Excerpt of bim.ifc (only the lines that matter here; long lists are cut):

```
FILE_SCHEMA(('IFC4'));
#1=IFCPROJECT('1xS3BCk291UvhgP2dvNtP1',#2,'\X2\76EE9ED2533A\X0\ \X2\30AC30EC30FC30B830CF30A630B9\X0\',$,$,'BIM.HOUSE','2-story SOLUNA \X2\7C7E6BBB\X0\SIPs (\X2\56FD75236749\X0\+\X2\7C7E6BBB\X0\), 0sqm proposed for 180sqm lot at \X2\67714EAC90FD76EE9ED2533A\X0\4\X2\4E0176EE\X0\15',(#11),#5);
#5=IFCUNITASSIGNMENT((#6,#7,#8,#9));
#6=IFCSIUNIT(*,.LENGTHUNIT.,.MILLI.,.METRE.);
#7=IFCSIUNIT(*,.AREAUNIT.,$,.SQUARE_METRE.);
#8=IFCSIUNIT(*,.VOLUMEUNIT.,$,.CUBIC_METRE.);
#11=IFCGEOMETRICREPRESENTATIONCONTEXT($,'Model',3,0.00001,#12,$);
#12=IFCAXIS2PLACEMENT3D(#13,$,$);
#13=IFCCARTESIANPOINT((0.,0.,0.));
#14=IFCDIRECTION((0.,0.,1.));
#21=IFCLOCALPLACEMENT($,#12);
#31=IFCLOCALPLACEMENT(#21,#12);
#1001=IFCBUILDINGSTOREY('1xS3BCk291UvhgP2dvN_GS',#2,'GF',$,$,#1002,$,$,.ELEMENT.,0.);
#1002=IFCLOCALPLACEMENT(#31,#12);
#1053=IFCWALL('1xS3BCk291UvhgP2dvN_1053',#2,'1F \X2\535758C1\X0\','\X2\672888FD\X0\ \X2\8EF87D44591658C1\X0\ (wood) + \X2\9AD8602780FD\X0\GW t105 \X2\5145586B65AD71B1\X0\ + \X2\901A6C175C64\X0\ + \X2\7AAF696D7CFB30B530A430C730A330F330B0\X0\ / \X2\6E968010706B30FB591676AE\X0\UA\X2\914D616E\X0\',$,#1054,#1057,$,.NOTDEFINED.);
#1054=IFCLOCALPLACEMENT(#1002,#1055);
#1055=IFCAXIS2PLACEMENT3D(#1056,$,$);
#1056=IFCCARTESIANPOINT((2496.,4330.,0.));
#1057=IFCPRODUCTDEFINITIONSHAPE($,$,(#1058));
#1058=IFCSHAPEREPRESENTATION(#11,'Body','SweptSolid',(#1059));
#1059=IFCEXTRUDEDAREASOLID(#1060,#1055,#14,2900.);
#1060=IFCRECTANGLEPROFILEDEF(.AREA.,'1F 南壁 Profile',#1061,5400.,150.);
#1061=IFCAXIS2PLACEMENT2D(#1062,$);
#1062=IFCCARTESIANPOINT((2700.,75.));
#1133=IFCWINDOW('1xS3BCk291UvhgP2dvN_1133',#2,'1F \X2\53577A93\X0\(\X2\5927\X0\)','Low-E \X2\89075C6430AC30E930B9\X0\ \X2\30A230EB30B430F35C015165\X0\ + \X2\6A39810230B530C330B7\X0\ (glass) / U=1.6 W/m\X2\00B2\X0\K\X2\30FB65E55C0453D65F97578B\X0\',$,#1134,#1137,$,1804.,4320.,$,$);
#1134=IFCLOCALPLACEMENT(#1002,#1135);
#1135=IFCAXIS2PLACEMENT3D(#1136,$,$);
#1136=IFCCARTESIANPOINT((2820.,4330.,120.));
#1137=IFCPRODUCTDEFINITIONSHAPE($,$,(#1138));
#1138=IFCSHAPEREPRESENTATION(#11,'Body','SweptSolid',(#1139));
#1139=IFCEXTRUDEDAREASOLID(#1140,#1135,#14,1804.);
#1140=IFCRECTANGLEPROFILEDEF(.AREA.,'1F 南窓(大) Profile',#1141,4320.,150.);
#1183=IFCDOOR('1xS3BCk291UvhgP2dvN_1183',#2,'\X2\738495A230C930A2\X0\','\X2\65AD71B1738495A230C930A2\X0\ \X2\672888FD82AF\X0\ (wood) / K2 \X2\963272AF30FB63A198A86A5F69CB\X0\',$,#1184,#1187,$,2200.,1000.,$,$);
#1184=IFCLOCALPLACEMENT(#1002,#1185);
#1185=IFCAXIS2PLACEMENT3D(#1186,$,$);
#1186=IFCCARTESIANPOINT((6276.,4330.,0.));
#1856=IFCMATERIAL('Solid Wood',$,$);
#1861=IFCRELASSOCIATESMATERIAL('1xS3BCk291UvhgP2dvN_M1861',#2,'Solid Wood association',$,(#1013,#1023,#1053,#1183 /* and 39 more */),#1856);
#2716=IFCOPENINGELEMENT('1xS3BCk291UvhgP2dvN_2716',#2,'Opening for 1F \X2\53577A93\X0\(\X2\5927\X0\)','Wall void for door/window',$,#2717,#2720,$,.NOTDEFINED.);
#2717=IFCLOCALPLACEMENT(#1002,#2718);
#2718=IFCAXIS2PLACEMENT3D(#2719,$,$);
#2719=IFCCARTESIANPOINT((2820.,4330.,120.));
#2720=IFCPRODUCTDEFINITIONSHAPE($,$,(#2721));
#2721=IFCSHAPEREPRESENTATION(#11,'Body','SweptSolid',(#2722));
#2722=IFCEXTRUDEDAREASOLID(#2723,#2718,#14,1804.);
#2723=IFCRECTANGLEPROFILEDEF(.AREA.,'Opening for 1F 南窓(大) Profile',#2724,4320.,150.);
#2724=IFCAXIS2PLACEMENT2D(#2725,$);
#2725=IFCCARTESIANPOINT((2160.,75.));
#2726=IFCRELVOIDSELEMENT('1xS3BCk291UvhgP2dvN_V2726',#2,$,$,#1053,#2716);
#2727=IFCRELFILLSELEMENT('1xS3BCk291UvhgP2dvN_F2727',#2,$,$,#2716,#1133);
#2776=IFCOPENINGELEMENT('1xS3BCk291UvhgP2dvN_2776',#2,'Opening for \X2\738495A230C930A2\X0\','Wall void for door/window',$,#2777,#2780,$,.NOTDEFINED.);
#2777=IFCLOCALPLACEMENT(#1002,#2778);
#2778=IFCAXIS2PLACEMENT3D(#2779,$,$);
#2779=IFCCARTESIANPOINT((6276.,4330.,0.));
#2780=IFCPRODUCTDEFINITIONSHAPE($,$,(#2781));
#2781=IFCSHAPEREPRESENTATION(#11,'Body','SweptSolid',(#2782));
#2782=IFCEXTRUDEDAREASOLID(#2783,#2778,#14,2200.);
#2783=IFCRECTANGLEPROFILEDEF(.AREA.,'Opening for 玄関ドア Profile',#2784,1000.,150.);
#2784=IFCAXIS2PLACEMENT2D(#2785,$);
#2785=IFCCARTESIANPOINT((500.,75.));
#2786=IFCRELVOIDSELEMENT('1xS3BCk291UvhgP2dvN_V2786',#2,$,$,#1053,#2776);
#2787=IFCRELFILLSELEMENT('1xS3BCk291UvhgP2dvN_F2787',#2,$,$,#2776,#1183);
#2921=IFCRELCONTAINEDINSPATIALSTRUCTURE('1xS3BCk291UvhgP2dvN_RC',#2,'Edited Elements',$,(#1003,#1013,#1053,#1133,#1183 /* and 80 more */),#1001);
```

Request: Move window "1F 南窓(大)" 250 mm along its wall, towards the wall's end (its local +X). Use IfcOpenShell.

```python
import ifcopenshell
import ifcopenshell.api.geometry
import ifcopenshell.util.placement

model = ifcopenshell.open("bim.ifc")

window = model.by_guid("1xS3BCk291UvhgP2dvN_1133")
opening = window.FillsVoids[0].RelatingOpeningElement
wall = opening.VoidsElements[0].RelatingBuildingElement

wall_matrix = ifcopenshell.util.placement.get_local_placement(wall.ObjectPlacement)
shift = wall_matrix[:3, 0] * 250.0
before = ifcopenshell.util.placement.get_local_placement(window.ObjectPlacement)[:3, 3].copy()

# The window is not placed relative to its opening, so move both.
for product in (opening, window):
    matrix = ifcopenshell.util.placement.get_local_placement(product.ObjectPlacement)
    matrix[:3, 3] += shift
    ifcopenshell.api.geometry.edit_object_placement(model, product=product, matrix=matrix, is_si=False)

after = ifcopenshell.util.placement.get_local_placement(window.ObjectPlacement)[:3, 3]
print("window moved by", (after - before).round(3) + 0.0)

model.write("bim_v2.ifc")
```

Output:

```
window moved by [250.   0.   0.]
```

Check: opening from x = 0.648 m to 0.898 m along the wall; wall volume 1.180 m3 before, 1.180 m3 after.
